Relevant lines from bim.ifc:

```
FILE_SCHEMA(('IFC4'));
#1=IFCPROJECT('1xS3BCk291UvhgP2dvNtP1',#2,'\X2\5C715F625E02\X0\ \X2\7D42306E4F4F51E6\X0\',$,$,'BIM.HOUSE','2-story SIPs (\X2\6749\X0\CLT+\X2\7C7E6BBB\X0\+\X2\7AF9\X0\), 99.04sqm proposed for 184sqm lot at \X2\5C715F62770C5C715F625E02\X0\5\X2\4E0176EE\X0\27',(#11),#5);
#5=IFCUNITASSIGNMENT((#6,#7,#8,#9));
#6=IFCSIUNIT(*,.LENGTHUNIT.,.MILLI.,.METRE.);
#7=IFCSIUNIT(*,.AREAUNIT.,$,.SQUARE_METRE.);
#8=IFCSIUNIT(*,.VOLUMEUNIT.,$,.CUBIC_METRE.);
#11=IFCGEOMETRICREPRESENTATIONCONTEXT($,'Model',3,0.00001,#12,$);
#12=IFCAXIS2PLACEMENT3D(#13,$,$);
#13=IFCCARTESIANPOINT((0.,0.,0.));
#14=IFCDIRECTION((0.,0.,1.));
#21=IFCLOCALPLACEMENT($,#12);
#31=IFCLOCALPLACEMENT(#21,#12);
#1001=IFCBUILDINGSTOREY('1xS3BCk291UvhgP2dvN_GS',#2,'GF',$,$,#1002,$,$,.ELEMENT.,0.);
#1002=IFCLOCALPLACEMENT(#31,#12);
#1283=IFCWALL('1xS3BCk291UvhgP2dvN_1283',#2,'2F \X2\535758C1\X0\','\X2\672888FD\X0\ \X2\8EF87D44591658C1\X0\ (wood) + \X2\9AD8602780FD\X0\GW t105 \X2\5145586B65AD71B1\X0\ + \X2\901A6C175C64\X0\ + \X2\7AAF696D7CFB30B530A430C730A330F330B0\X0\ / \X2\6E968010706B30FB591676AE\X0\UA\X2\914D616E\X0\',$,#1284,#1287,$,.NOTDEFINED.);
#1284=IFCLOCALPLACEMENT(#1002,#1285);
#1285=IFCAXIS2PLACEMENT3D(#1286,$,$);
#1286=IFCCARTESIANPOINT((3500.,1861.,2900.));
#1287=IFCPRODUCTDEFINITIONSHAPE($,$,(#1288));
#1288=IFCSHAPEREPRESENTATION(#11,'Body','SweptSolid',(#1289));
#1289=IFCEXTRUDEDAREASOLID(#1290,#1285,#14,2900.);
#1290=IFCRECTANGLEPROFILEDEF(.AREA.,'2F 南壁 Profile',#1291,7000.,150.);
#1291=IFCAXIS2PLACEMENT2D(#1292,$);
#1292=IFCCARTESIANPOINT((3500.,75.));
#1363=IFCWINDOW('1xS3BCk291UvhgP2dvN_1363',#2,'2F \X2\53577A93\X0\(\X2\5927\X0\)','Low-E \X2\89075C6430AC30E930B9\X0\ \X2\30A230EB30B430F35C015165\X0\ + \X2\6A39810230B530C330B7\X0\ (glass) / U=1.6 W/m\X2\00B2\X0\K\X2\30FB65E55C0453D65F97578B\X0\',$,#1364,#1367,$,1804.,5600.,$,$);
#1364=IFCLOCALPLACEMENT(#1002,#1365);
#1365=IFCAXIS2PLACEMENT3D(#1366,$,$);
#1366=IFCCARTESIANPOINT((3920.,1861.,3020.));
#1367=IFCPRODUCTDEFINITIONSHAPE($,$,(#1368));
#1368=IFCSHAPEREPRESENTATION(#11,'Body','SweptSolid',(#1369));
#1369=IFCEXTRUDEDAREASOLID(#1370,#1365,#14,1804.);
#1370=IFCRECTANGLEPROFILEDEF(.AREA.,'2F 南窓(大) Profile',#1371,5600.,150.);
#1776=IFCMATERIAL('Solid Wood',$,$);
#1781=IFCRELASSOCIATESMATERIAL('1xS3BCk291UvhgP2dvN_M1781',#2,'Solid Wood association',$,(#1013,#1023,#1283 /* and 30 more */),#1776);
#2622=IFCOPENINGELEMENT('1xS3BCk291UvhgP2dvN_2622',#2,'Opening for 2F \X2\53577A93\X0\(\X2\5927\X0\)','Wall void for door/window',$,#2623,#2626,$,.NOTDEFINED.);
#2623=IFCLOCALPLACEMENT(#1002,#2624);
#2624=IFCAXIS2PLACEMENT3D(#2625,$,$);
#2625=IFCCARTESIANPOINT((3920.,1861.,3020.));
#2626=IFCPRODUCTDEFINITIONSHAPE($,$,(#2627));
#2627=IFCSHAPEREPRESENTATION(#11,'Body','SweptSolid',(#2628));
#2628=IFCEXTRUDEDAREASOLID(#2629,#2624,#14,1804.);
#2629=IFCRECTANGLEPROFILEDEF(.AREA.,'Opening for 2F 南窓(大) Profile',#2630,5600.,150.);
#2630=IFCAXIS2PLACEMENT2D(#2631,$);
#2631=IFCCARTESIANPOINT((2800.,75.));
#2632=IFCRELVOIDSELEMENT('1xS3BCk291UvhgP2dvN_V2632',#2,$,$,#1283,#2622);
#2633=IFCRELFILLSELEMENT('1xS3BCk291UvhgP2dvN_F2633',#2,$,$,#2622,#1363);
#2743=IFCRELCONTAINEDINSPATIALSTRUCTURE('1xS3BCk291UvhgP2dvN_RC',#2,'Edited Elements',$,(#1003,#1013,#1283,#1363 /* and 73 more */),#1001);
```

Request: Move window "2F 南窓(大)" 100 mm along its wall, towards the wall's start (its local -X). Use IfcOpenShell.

```python
import ifcopenshell
import ifcopenshell.api.geometry
import ifcopenshell.util.placement
import ifcopenshell.util.unit

model = ifcopenshell.open("bim.ifc")
unit_scale = ifcopenshell.util.unit.calculate_unit_scale(model)

window = model.by_id(1363)
opening = window.FillsVoids[0].RelatingOpeningElement
wall = opening.VoidsElements[0].RelatingBuildingElement

wall_matrix = ifcopenshell.util.placement.get_local_placement(wall.ObjectPlacement)
shift = wall_matrix[:3, 0] * -0.1 / unit_scale
before = ifcopenshell.util.placement.get_local_placement(window.ObjectPlacement)[:3, 3].copy()

# The window is not placed relative to its opening, so move both.
for product in (opening, window):
    matrix = ifcopenshell.util.placement.get_local_placement(product.ObjectPlacement)
    matrix[:3, 3] += shift
    ifcopenshell.api.geometry.edit_object_placement(model, product=product, matrix=matrix, is_si=False)

after = ifcopenshell.util.placement.get_local_placement(window.ObjectPlacement)[:3, 3]
print("window moved by", (after - before).round(3) + 0.0)

model.write("bim_v2.ifc")
```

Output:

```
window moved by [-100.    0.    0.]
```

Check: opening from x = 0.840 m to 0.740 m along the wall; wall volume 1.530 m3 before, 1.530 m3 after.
